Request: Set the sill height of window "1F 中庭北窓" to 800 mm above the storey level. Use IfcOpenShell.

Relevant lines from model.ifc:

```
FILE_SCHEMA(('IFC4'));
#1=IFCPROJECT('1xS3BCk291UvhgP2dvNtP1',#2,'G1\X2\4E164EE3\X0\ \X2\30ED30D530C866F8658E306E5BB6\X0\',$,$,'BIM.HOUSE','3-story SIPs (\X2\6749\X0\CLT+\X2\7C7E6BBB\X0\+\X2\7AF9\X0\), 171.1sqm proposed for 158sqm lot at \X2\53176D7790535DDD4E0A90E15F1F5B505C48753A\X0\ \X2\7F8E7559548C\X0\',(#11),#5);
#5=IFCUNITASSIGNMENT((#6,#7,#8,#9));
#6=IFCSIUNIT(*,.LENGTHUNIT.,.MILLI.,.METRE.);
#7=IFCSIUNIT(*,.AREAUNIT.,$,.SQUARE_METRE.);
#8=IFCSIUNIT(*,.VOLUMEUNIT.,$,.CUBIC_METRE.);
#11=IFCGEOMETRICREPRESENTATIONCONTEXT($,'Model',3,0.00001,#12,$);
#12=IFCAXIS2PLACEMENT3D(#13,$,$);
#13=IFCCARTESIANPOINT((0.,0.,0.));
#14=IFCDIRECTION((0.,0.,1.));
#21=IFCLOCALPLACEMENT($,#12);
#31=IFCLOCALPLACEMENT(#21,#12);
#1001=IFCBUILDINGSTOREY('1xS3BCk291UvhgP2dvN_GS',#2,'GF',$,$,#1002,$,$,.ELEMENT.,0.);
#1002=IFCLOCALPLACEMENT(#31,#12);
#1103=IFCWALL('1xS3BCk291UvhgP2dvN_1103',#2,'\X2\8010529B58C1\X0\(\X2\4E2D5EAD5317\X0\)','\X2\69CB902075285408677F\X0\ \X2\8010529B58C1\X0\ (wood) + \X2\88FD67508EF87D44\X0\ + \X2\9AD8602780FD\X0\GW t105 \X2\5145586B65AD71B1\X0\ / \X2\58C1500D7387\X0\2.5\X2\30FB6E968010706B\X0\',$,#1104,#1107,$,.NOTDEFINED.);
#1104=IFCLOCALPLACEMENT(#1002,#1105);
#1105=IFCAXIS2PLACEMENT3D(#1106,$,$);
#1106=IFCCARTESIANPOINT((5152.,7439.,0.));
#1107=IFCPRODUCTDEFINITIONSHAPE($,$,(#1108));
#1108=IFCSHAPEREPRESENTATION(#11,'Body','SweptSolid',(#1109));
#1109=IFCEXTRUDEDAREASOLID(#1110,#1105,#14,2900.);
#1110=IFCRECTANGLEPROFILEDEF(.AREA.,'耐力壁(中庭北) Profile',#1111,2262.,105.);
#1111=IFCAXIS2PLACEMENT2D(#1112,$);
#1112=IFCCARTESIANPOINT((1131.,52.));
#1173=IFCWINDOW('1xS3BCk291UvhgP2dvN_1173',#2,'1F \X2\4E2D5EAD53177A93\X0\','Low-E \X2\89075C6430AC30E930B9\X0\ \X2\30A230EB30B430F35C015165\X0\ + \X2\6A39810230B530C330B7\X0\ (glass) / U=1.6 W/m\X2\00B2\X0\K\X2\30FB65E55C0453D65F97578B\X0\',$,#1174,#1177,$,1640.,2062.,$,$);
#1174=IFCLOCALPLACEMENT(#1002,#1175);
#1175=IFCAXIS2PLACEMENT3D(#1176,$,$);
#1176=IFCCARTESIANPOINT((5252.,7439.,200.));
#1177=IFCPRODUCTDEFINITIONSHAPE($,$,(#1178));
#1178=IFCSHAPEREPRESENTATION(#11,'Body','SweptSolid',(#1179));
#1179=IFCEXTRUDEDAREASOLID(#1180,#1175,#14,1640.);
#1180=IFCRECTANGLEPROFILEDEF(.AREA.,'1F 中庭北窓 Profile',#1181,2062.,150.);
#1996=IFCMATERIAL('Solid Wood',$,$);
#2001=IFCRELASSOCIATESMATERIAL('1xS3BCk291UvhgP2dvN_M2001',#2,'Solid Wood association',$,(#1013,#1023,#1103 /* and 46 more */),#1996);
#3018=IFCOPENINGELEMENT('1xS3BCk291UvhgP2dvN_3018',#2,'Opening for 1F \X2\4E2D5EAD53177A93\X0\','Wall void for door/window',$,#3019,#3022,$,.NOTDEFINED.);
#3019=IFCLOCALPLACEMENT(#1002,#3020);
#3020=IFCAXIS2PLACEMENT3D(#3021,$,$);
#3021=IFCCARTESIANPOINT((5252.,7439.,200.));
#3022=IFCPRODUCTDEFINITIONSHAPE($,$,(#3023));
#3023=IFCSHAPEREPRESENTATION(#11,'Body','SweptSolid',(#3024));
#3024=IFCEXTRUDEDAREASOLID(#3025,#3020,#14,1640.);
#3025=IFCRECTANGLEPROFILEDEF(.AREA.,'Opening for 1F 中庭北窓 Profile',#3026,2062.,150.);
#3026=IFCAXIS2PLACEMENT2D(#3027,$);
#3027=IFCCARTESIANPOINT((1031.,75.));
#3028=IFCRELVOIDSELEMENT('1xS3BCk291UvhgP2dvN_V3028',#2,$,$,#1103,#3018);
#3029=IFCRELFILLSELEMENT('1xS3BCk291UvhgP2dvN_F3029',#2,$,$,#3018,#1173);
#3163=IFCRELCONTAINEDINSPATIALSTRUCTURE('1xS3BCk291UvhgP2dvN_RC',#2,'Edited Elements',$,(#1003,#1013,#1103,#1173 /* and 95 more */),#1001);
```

```python
import numpy as np
import ifcopenshell
import ifcopenshell.api.geometry
import ifcopenshell.geom
import ifcopenshell.util.element
import ifcopenshell.util.placement
import ifcopenshell.util.shape
import ifcopenshell.util.unit

model = ifcopenshell.open("model.ifc")
unit_scale = ifcopenshell.util.unit.calculate_unit_scale(model)

window = model.by_guid("1xS3BCk291UvhgP2dvN_1173")
opening = window.FillsVoids[0].RelatingOpeningElement
storey = ifcopenshell.util.element.get_container(window, ifc_class="IfcBuildingStorey")
level = ifcopenshell.util.placement.get_local_placement(storey.ObjectPlacement)[2, 3]

# The opening's origin need not be at the sill, so measure its lowest point.
shape = ifcopenshell.geom.create_shape(ifcopenshell.geom.settings(), opening)
bottom = ifcopenshell.util.shape.get_shape_bottom_elevation(shape, shape.geometry) / unit_scale
dz = level + 0.8 / unit_scale - bottom

shift = np.array([0.0, 0.0, dz])
# The window is not placed relative to its opening, so move both.
for product in (opening, window):
    matrix = ifcopenshell.util.placement.get_local_placement(product.ObjectPlacement)
    matrix[:3, 3] += shift
    ifcopenshell.api.geometry.edit_object_placement(model, product=product, matrix=matrix, is_si=False)

print(f"moved by {dz * unit_scale:+.3f} m")

model.write("model_rev.ifc")
```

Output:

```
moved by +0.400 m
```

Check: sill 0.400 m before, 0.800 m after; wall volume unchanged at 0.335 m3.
